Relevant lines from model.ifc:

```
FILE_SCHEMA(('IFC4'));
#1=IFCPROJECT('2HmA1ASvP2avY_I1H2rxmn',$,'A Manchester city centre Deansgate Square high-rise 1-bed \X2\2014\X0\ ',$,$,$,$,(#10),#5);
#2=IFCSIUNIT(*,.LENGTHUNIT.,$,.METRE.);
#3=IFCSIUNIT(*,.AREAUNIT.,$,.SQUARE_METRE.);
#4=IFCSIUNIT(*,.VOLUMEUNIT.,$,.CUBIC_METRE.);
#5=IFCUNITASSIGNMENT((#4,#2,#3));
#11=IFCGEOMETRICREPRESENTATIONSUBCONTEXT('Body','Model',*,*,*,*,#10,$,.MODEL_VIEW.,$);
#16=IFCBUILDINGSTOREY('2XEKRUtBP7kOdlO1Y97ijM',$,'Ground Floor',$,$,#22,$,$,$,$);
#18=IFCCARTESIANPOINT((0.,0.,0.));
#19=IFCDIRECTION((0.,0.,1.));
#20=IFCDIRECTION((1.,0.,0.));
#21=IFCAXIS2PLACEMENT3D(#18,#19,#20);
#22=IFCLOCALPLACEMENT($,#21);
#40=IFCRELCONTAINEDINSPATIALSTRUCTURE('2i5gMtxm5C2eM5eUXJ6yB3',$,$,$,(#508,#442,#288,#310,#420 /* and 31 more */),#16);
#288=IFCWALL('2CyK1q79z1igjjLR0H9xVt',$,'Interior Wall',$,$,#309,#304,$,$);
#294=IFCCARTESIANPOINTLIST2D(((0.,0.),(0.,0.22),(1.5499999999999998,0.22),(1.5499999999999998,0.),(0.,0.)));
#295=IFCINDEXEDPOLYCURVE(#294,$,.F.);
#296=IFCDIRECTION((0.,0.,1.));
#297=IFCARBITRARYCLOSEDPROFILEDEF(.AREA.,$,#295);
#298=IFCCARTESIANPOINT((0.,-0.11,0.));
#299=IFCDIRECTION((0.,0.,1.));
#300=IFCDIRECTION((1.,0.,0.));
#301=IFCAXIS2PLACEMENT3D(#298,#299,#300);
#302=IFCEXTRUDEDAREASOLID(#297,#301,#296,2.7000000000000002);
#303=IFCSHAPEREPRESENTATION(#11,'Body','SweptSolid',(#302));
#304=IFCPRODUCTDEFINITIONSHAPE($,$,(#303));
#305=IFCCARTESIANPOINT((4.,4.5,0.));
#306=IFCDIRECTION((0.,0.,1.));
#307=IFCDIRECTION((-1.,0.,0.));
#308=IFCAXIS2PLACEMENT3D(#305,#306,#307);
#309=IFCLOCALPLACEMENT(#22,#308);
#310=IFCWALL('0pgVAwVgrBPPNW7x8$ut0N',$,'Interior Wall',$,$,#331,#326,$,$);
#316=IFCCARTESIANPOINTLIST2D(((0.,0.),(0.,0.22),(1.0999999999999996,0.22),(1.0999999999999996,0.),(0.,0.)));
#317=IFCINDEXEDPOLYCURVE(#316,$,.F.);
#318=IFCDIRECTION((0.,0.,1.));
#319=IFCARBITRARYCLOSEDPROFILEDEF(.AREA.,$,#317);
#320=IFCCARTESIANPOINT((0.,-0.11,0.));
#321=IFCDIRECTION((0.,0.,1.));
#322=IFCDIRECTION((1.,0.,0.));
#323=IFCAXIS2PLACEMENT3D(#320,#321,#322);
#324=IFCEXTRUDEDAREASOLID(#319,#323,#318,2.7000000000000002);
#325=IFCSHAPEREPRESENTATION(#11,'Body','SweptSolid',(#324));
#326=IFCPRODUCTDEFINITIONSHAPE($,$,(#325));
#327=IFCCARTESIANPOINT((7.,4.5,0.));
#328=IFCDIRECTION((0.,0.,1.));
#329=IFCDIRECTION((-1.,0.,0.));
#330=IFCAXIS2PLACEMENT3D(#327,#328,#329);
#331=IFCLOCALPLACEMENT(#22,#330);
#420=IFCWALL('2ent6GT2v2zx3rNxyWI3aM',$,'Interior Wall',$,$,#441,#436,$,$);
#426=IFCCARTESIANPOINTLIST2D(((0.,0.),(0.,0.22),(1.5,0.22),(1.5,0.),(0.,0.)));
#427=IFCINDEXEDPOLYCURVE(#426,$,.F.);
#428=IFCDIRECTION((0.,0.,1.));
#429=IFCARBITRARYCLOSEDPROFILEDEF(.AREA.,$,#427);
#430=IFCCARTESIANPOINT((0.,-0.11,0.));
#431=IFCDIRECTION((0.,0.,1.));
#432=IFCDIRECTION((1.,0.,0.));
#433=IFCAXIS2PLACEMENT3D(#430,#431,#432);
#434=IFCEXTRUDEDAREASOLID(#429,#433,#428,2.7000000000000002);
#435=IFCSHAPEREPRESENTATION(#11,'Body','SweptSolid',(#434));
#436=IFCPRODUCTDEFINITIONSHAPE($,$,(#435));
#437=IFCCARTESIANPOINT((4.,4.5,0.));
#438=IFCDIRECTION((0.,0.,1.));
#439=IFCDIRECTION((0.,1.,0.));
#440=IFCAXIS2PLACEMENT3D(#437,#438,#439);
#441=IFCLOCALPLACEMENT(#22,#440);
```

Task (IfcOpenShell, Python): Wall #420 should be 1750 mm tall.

```python
import ifcopenshell
import ifcopenshell.geom
import ifcopenshell.util.representation
import ifcopenshell.util.shape
import ifcopenshell.util.unit

model = ifcopenshell.open("model.ifc")
unit_scale = ifcopenshell.util.unit.calculate_unit_scale(model)
settings = ifcopenshell.geom.settings()


def volume(element):
    """Net volume in cubic metres, openings subtracted."""
    shape = ifcopenshell.geom.create_shape(settings, element)
    return ifcopenshell.util.shape.get_volume(shape.geometry)


wall = model.by_guid("2ent6GT2v2zx3rNxyWI3aM")
before = volume(wall)

body = ifcopenshell.util.representation.get_representation(wall, "Model", "Body")
solid = body.Items[0]
old_height = solid.Depth
solid.Depth = 1.75 / unit_scale
after = volume(wall)

print(f"height {old_height:g} -> {solid.Depth:g}, volume {before:.3f} -> {after:.3f} m3")

model.write("model_updated.ifc")
```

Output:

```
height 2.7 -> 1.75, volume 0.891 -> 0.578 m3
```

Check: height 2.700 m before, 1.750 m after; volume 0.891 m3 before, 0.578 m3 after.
